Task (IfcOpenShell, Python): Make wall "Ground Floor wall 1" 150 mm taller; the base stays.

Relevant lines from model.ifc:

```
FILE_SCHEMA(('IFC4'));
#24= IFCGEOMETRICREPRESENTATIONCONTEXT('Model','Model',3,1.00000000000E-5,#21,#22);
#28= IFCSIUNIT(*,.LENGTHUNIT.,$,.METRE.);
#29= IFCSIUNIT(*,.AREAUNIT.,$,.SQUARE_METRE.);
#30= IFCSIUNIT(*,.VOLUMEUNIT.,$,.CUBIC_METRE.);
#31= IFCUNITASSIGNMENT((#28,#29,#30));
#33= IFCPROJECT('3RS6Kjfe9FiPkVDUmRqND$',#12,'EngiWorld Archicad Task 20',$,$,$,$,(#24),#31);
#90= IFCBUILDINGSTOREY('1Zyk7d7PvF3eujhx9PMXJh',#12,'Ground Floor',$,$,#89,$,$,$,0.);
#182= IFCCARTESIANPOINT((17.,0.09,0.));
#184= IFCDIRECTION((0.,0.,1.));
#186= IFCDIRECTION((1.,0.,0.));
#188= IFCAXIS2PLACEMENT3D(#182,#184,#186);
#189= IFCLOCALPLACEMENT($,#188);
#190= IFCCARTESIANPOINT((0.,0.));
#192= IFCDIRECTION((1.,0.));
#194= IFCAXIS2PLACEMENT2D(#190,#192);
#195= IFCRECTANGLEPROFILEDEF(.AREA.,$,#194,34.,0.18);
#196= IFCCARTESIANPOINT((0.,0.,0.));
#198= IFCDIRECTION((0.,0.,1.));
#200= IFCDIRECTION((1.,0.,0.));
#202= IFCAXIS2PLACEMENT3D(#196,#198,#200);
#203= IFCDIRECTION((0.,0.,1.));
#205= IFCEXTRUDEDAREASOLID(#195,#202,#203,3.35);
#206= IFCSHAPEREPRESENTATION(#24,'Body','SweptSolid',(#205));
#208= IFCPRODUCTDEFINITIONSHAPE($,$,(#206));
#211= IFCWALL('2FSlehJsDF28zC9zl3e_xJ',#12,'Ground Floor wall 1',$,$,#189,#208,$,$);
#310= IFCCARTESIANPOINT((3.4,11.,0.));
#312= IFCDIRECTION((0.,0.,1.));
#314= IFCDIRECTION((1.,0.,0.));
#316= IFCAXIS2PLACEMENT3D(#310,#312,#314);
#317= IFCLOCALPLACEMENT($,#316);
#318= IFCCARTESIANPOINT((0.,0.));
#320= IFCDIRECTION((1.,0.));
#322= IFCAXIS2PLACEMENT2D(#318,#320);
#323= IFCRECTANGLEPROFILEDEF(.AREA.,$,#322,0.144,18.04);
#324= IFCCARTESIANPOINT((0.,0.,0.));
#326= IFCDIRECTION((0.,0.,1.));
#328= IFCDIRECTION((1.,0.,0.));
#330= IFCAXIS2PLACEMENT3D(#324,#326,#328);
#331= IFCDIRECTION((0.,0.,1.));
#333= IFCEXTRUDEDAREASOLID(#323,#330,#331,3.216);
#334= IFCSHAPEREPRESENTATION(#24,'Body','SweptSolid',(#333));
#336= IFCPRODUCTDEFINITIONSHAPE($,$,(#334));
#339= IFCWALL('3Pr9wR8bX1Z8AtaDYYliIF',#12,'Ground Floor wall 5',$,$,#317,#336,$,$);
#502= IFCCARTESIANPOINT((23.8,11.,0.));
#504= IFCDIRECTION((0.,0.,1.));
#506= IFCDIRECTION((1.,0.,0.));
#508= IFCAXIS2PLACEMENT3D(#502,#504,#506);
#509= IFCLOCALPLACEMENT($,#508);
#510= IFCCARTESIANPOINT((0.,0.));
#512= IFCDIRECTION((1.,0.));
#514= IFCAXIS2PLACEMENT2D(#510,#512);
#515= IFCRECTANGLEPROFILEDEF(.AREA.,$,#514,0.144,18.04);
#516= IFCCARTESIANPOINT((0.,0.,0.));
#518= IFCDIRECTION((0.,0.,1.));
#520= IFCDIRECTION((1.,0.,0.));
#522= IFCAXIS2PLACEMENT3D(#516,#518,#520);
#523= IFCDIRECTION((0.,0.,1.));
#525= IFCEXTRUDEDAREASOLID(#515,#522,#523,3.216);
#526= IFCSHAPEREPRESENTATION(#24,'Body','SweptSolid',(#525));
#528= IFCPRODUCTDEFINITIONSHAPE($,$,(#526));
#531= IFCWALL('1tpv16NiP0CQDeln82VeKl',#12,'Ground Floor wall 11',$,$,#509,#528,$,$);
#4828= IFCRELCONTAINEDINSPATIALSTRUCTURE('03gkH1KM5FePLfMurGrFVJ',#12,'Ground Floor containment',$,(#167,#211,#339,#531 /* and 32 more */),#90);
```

```python
import ifcopenshell
import ifcopenshell.geom
import ifcopenshell.util.shape
import ifcopenshell.util.unit

model = ifcopenshell.open("model.ifc")
unit_scale = ifcopenshell.util.unit.calculate_unit_scale(model)
settings = ifcopenshell.geom.settings()


def volume(element):
    """Net volume in cubic metres, openings subtracted."""
    shape = ifcopenshell.geom.create_shape(settings, element)
    return ifcopenshell.util.shape.get_volume(shape.geometry)


wall = model.by_id(211)
before = volume(wall)

body = next(r for r in wall.Representation.Representations if r.RepresentationIdentifier == "Body")
solid = body.Items[0]
old_height = solid.Depth
solid.Depth += 0.15 / unit_scale
after = volume(wall)

print(f"height {old_height:g} -> {solid.Depth:g}, volume {before:.3f} -> {after:.3f} m3")

model.write("model_rev.ifc")
```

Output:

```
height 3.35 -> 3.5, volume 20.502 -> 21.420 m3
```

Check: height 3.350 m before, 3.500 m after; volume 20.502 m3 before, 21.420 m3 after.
